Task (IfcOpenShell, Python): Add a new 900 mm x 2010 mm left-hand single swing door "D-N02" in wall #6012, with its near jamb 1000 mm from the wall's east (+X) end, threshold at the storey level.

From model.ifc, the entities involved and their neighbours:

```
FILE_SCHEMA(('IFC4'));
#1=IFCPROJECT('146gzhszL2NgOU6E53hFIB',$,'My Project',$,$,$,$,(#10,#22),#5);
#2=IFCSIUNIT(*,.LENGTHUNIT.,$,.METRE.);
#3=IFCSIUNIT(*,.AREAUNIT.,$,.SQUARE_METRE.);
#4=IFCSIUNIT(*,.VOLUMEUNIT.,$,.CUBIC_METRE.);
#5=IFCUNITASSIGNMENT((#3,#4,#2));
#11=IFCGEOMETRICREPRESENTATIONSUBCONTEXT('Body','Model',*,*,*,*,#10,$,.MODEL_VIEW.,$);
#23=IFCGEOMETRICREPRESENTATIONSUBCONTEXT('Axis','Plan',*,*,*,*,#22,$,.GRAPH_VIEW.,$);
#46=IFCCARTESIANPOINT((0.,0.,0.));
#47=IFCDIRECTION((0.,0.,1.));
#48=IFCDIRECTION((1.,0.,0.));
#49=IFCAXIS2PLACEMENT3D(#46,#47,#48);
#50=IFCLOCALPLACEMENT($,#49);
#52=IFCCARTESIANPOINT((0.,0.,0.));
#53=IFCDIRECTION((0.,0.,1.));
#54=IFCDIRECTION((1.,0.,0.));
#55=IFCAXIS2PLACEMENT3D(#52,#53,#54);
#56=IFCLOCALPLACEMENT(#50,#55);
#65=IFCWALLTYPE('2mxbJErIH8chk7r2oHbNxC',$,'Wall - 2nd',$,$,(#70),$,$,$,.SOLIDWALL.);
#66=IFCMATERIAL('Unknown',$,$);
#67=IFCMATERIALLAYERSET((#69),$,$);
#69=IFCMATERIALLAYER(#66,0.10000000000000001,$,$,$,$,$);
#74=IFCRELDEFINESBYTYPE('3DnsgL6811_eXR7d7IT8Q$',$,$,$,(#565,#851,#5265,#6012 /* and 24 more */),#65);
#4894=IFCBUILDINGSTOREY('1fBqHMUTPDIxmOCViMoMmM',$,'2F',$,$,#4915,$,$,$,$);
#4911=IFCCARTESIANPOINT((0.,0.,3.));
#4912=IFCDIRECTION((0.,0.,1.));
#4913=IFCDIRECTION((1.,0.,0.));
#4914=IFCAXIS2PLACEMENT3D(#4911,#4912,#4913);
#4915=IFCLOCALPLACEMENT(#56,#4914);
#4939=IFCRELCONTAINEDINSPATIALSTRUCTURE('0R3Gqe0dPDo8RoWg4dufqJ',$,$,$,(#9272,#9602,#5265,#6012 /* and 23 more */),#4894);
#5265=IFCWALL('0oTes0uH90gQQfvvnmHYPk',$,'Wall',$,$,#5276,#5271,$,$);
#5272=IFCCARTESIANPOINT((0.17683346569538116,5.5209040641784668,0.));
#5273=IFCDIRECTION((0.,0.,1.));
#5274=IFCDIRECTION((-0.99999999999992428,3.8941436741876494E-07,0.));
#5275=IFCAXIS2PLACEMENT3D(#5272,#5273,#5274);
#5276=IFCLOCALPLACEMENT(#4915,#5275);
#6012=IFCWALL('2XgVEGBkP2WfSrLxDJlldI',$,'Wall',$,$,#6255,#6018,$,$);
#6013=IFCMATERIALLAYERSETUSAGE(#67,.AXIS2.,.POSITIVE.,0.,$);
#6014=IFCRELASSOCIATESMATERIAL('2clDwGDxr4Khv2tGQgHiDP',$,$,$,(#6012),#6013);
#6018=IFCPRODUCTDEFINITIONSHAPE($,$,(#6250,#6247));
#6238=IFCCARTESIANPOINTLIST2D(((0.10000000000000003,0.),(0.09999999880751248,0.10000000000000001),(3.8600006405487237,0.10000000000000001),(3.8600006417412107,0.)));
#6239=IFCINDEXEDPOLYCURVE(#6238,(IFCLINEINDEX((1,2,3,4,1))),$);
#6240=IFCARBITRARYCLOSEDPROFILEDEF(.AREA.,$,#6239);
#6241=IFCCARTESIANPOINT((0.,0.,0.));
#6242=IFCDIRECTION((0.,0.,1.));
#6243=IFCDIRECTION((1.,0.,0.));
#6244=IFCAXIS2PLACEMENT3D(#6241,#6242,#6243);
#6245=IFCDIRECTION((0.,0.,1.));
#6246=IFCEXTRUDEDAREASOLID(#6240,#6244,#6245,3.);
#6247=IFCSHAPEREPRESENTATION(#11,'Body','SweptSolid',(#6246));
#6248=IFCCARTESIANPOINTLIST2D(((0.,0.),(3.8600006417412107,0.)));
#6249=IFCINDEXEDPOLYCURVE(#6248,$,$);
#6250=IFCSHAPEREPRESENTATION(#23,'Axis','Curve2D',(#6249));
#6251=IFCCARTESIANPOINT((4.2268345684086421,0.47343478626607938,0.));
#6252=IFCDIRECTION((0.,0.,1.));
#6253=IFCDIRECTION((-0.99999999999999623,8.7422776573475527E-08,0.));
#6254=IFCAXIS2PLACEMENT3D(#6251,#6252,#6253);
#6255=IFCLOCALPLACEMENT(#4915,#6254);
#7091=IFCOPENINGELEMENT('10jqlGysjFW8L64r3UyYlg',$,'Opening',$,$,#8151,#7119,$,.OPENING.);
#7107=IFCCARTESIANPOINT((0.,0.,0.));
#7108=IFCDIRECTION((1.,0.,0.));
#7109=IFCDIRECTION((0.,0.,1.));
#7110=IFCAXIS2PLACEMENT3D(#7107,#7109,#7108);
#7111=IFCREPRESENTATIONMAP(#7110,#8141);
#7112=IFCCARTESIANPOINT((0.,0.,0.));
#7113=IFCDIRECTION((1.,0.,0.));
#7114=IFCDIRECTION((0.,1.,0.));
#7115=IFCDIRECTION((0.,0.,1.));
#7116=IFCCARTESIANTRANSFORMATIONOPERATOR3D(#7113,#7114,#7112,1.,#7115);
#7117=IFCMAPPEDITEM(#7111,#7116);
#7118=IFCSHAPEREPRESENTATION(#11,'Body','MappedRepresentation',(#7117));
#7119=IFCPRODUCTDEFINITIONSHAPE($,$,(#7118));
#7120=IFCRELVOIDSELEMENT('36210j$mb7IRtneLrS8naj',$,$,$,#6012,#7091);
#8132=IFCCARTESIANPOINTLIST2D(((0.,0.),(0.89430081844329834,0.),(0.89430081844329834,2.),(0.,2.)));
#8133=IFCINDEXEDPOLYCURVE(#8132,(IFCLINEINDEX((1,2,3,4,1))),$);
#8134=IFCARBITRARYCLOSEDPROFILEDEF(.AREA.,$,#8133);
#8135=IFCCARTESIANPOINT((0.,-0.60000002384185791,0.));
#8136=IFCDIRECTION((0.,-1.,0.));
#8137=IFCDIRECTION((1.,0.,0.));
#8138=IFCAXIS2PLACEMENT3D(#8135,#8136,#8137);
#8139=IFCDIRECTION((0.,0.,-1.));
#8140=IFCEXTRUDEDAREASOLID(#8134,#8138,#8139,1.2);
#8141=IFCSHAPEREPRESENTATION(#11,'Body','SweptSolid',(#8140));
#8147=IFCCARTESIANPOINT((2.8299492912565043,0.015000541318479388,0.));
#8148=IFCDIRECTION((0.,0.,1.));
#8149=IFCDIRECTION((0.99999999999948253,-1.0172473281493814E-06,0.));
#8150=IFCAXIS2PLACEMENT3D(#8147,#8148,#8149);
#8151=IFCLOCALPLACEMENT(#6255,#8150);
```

```python
import numpy as np
import ifcopenshell
import ifcopenshell.api.feature
import ifcopenshell.api.geometry
import ifcopenshell.api.root
import ifcopenshell.api.spatial
import ifcopenshell.geom
import ifcopenshell.util.element
import ifcopenshell.util.placement
import ifcopenshell.util.representation
import ifcopenshell.util.shape
import ifcopenshell.util.unit

model = ifcopenshell.open("model.ifc")
unit_scale = ifcopenshell.util.unit.calculate_unit_scale(model)
settings = ifcopenshell.geom.settings()


def volume(element):
    """Net volume in cubic metres, openings subtracted."""
    shape = ifcopenshell.geom.create_shape(settings, element)
    return ifcopenshell.util.shape.get_volume(shape.geometry)


wall = model.by_guid("2XgVEGBkP2WfSrLxDJlldI")
storey = ifcopenshell.util.element.get_container(wall, ifc_class="IfcBuildingStorey")
context = ifcopenshell.util.representation.get_context(model, "Model", "Body", "MODEL_VIEW")
before = volume(wall)

width, height, from_end, sill = 0.9, 2.01, 1, 0.0  # metres

# The wall runs along its own X axis, and the end named is its -X end.
wall_shape = ifcopenshell.geom.create_shape(settings, wall)
x, y, z = ifcopenshell.util.shape.get_vertices(wall_shape.geometry).T
start = x.min() + from_end
face, thickness = float(y.min()), float(y.max() - y.min())
wall_matrix = ifcopenshell.util.placement.get_local_placement(wall.ObjectPlacement)
level = ifcopenshell.util.placement.get_local_placement(storey.ObjectPlacement)[2, 3]


def in_wall(x, y):
    """Placement at x, y metres in the wall's axes, at sill height."""
    matrix = wall_matrix.copy()
    matrix[:, 3] = wall_matrix @ np.array([x / unit_scale, y / unit_scale, 0.0, 1.0])
    matrix[2, 3] = level + sill / unit_scale
    return matrix


# Opening: a box that overshoots both wall faces by 50 mm.
opening = ifcopenshell.api.root.create_entity(model, ifc_class="IfcOpeningElement", predefined_type="OPENING")
box = ifcopenshell.api.geometry.add_wall_representation(
    model, context=context, length=width, height=height, thickness=thickness + 0.1
)
ifcopenshell.api.geometry.assign_representation(model, product=opening, representation=box)
ifcopenshell.api.geometry.edit_object_placement(model, product=opening, matrix=in_wall(start, face - 0.05), is_si=False)
ifcopenshell.api.feature.add_feature(model, feature=opening, element=wall)

door = ifcopenshell.api.root.create_entity(model, ifc_class="IfcDoor", name="D-N02", predefined_type="DOOR")
door.OverallWidth, door.OverallHeight = width / unit_scale, height / unit_scale
door.OperationType = "SINGLE_SWING_LEFT"
body = ifcopenshell.api.geometry.add_door_representation(
    model,
    context=context,
    overall_width=door.OverallWidth,
    overall_height=door.OverallHeight,
    operation_type="SINGLE_SWING_LEFT",
    lining_properties={"LiningDepth": thickness / unit_scale, "ThresholdDepth": thickness / unit_scale},
)
ifcopenshell.api.geometry.assign_representation(model, product=door, representation=body)
ifcopenshell.api.spatial.assign_container(model, products=[door], relating_structure=storey)
ifcopenshell.api.feature.add_filling(model, opening=opening, element=door)

# The lining spans the wall, so the door starts at the wall face.
ifcopenshell.api.geometry.edit_object_placement(model, product=door, matrix=in_wall(start, face), is_si=False)

after = volume(wall)

print(f"wall volume {before:.3f} -> {after:.3f} m3")

model.write("model_v2.ifc")
```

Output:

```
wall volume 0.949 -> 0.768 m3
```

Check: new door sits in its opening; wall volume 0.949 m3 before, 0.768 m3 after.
